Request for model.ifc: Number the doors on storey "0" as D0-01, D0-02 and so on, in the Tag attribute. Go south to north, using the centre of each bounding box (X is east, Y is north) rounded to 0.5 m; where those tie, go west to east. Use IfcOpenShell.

First a look at what the model holds.

```python
import ifcopenshell
import ifcopenshell.util.element
import ifcopenshell.util.placement

model = ifcopenshell.open("model.ifc")
print(model.schema)
storey = next(s for s in model.by_type("IfcBuildingStorey") if s.Name == "0")
doors = [e for e in ifcopenshell.util.element.get_decomposition(storey) if e.is_a("IfcDoor")]
for e in sorted(doors, key=lambda e: e.id()):
    origin = ifcopenshell.util.placement.get_local_placement(e.ObjectPlacement)[:3, 3]
    print(e.id(), e.Tag, e.Name, origin.round(2) + 0.0, sep=" | ")
```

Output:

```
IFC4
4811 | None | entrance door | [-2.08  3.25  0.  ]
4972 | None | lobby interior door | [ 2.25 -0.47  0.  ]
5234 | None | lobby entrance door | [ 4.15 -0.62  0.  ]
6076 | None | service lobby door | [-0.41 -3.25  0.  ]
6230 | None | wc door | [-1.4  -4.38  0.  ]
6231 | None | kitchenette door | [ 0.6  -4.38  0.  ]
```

```python
import ifcopenshell
import ifcopenshell.geom
import ifcopenshell.util.element
import ifcopenshell.util.shape

model = ifcopenshell.open("model.ifc")
settings = ifcopenshell.geom.settings()
settings.set("use-world-coords", True)


def centre(element):
    shape = ifcopenshell.geom.create_shape(settings, element)
    return ifcopenshell.util.shape.get_bbox_centroid(shape.geometry)


storey = next(s for s in model.by_type("IfcBuildingStorey") if s.Name == "0")
doors = [e for e in ifcopenshell.util.element.get_decomposition(storey) if e.is_a("IfcDoor")]

# Insertion points can sit at a corner or the storey origin, so sort by the geometry (in metres).
centres = {e: centre(e) for e in doors}
doors.sort(key=lambda e: (round(centres[e][1] / 0.5), centres[e][0]))

for i, e in enumerate(doors, start=1):
    number = f"D0-{i:02d}"
    e.Tag = number
    print(e.id(), number)

model.write("model_rev.ifc")
```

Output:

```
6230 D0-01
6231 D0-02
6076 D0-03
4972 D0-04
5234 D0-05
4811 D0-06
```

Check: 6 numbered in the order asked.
